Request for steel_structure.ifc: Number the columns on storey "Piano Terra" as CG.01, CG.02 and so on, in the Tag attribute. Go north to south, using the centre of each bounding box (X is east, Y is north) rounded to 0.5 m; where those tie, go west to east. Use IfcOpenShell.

First a look at what the model holds.

```python
import ifcopenshell
import ifcopenshell.util.element
import ifcopenshell.util.placement

model = ifcopenshell.open("steel_structure.ifc")
print(model.schema)
storey = next(s for s in model.by_type("IfcBuildingStorey") if s.Name == "Piano Terra")
columns = [e for e in ifcopenshell.util.element.get_decomposition(storey) if e.is_a("IfcColumn")]
for e in sorted(columns, key=lambda e: e.id()):
    origin = ifcopenshell.util.placement.get_local_placement(e.ObjectPlacement)[:3, 3]
    print(e.id(), e.Tag, e.Name, origin.round(2) + 0.0, sep=" | ")
```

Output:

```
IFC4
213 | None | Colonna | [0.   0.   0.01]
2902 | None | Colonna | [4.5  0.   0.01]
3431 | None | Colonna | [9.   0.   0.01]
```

```python
import ifcopenshell
import ifcopenshell.geom
import ifcopenshell.util.element
import ifcopenshell.util.shape

model = ifcopenshell.open("steel_structure.ifc")
settings = ifcopenshell.geom.settings()
settings.set("use-world-coords", True)


def centre(element):
    shape = ifcopenshell.geom.create_shape(settings, element)
    return ifcopenshell.util.shape.get_bbox_centroid(shape.geometry)


storey = next(s for s in model.by_type("IfcBuildingStorey") if s.Name == "Piano Terra")
columns = [e for e in ifcopenshell.util.element.get_decomposition(storey) if e.is_a("IfcColumn")]

# Insertion points can sit at a corner or the storey origin, so sort by the geometry (in metres).
centres = {e: centre(e) for e in columns}
columns.sort(key=lambda e: (-round(centres[e][1] / 0.5), centres[e][0]))

for i, e in enumerate(columns, start=1):
    number = f"CG.{i:02d}"
    e.Tag = number
    print(e.id(), number)

model.write("steel_structure-out.ifc")
```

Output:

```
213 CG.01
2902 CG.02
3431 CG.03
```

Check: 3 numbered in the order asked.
